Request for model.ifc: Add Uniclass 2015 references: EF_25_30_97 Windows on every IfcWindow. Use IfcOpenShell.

First a look at what the model holds.

```python
import ifcopenshell

model = ifcopenshell.open("model.ifc")
print(model.schema)
print("classifications:", [c.Name for c in model.by_type("IfcClassification")])
for ifc_class in ("IfcDoor", "IfcRoof", "IfcStair", "IfcWall", "IfcWindow"):
    print(ifc_class, len(model.by_type(ifc_class)))
```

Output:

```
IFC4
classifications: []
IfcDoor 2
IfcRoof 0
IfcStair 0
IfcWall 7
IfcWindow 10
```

```python
import ifcopenshell
import ifcopenshell.api.classification

model = ifcopenshell.open("model.ifc")

system = ifcopenshell.api.classification.add_classification(model, classification="Uniclass 2015")

codes = {
    "IfcWindow": ("EF_25_30_97", "Windows"),
}
for ifc_class, (code, name) in codes.items():
    products = model.by_type(ifc_class)
    ifcopenshell.api.classification.add_reference(
        model, products=products, classification=system, identification=code, name=name
    )
    print(code, len(products))

model.write("model_v2.ifc")
```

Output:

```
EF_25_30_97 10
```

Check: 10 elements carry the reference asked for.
